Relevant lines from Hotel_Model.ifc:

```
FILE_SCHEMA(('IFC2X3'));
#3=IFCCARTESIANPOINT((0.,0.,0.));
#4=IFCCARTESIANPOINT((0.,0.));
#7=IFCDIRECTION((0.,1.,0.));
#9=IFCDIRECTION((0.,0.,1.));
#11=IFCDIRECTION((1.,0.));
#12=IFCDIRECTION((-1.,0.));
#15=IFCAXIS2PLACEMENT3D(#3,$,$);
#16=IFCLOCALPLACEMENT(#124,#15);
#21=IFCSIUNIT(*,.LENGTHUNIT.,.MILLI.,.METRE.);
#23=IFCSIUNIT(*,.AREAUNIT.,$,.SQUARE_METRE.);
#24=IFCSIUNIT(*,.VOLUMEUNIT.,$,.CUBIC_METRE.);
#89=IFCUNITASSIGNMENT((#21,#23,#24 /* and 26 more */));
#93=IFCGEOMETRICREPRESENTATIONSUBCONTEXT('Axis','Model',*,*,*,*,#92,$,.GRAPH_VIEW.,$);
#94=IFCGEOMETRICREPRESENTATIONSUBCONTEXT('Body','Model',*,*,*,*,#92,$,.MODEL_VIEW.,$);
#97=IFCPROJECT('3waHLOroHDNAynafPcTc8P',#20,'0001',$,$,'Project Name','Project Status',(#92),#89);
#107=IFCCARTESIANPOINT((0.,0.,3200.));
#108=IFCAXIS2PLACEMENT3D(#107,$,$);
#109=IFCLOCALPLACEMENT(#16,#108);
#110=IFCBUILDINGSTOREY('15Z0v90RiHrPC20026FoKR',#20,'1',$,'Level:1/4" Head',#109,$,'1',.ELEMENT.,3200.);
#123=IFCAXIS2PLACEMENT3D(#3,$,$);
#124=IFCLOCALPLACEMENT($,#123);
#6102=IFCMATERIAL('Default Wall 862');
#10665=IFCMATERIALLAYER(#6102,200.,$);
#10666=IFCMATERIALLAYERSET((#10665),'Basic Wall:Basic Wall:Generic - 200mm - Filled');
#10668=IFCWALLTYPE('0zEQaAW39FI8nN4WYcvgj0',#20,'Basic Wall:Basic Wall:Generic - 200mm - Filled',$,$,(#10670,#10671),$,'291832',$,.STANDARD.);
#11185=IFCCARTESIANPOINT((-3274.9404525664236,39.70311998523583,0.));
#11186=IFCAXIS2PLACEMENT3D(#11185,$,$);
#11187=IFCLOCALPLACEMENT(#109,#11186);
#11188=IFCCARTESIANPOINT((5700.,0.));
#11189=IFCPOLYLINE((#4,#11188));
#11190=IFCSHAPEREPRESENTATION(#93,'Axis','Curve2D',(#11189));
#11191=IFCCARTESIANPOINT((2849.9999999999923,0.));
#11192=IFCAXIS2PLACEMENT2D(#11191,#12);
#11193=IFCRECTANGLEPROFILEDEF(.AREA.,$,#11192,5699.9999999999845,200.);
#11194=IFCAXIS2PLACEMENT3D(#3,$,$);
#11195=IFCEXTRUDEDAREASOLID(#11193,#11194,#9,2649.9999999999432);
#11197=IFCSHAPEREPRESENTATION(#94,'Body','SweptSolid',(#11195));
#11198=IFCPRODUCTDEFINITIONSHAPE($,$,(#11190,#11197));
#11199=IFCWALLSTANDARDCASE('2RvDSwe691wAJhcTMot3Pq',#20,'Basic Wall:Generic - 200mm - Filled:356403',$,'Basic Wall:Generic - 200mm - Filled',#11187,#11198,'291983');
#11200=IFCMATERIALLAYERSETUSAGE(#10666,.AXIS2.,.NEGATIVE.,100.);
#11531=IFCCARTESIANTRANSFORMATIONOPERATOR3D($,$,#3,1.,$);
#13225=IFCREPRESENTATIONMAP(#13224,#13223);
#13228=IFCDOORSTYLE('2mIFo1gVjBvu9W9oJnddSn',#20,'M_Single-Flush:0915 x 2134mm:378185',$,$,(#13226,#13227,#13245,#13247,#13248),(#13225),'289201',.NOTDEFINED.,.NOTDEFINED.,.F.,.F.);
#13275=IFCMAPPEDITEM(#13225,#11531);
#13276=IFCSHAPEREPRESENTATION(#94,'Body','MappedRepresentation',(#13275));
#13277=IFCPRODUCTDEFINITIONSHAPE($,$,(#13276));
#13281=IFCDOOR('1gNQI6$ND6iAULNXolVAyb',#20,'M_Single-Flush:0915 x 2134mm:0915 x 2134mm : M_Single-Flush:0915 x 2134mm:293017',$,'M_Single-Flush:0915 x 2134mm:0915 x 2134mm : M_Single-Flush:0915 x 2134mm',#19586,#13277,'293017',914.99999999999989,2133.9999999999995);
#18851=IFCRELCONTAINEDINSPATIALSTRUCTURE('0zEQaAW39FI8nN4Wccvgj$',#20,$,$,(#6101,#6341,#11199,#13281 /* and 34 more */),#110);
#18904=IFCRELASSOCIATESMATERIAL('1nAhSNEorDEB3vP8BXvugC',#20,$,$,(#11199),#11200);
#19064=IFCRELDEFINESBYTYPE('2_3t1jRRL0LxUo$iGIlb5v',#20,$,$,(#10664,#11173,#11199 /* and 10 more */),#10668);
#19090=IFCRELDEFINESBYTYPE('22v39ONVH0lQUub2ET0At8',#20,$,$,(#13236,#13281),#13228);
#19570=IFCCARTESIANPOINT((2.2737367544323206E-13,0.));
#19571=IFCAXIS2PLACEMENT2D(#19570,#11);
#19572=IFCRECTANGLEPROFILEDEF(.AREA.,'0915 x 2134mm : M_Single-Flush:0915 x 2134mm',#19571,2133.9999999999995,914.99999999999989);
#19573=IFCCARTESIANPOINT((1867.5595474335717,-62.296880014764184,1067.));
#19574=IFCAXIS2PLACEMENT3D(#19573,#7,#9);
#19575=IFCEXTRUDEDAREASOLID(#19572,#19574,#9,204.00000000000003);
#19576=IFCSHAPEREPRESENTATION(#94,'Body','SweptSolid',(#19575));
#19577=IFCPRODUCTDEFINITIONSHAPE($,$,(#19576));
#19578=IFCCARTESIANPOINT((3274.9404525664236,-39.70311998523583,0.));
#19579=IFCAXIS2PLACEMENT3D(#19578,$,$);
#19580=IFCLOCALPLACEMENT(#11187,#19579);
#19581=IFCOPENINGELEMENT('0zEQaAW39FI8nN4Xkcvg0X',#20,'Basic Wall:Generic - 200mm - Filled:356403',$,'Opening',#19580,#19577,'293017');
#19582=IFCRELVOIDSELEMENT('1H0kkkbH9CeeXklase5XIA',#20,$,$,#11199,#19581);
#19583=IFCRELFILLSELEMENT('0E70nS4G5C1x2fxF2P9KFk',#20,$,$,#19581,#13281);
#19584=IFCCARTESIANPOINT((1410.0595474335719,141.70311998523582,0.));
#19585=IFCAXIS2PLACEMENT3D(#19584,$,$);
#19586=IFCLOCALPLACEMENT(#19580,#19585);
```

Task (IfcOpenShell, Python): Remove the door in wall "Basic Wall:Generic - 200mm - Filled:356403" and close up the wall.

```python
import ifcopenshell
import ifcopenshell.api.feature
import ifcopenshell.api.root
import ifcopenshell.geom
import ifcopenshell.util.shape

model = ifcopenshell.open("Hotel_Model.ifc")
settings = ifcopenshell.geom.settings()


def volume(element):
    """Net volume in cubic metres, openings subtracted."""
    shape = ifcopenshell.geom.create_shape(settings, element)
    return ifcopenshell.util.shape.get_volume(shape.geometry)


door = model.by_guid("1gNQI6$ND6iAULNXolVAyb")
opening = door.FillsVoids[0].RelatingOpeningElement
wall = opening.VoidsElements[0].RelatingBuildingElement
before = volume(wall)

ifcopenshell.api.root.remove_product(model, product=door)
ifcopenshell.api.feature.remove_feature(model, feature=opening)

after = volume(wall)

print(f"wall volume {before:.3f} -> {after:.3f} m3")

model.write("Hotel_Model_v2.ifc")
```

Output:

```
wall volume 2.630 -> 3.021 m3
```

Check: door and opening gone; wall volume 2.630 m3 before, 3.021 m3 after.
